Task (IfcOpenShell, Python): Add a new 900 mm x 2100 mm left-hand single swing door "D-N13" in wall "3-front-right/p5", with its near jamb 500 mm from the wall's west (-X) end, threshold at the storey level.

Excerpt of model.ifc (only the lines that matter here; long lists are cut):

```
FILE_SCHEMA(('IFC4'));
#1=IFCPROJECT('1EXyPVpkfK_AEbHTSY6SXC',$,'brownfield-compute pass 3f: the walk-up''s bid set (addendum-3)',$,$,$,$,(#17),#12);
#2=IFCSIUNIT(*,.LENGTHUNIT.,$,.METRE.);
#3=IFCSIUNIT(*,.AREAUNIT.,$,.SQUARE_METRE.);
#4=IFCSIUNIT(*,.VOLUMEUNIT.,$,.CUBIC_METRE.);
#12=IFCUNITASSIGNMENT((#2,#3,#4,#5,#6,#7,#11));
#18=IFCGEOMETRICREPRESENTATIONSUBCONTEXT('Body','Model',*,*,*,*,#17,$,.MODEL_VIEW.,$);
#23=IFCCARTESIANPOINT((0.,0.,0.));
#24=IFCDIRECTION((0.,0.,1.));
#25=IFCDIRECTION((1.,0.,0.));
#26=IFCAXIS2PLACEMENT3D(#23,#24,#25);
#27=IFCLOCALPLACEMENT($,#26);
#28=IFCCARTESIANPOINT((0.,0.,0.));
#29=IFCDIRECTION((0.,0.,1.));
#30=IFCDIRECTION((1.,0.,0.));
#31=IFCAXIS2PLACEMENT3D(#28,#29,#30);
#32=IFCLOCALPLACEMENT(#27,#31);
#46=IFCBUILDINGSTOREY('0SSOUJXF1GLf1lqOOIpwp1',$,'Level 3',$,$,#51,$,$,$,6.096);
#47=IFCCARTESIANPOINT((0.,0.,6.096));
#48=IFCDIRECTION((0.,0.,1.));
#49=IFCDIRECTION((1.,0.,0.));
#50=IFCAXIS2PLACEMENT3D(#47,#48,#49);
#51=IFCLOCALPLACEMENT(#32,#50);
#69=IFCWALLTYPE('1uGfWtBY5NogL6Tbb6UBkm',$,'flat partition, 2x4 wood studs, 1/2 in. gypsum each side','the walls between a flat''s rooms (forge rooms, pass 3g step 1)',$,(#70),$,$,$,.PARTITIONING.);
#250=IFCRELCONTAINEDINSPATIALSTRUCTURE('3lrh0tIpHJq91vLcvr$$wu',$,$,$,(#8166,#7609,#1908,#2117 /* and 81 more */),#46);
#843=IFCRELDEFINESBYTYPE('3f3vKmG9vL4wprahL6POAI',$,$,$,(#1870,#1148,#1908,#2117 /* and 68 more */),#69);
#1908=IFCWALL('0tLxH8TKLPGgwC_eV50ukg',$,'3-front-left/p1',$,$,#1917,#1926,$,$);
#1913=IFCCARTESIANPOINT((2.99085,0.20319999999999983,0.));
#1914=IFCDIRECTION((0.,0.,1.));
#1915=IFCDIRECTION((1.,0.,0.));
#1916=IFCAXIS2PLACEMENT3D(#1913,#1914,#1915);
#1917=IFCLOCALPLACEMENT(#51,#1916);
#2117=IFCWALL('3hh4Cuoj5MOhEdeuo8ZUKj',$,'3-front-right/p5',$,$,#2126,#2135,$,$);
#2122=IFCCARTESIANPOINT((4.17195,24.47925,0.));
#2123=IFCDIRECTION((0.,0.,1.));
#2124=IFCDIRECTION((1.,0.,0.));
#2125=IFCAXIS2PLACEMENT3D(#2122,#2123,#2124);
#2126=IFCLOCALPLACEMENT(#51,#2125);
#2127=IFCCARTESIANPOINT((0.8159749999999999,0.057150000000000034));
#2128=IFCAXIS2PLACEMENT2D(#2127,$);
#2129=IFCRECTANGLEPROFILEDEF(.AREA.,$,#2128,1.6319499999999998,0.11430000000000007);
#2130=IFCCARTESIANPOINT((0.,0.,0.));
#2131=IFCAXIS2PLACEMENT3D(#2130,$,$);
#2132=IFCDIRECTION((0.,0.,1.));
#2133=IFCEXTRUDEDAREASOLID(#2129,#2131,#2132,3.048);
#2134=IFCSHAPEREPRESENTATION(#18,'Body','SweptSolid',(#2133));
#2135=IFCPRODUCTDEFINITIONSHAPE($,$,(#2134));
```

```python
import numpy as np
import ifcopenshell
import ifcopenshell.api.feature
import ifcopenshell.api.geometry
import ifcopenshell.api.root
import ifcopenshell.api.spatial
import ifcopenshell.geom
import ifcopenshell.util.element
import ifcopenshell.util.placement
import ifcopenshell.util.representation
import ifcopenshell.util.shape
import ifcopenshell.util.unit

model = ifcopenshell.open("model.ifc")
unit_scale = ifcopenshell.util.unit.calculate_unit_scale(model)
settings = ifcopenshell.geom.settings()


def volume(element):
    """Net volume in cubic metres, openings subtracted."""
    shape = ifcopenshell.geom.create_shape(settings, element)
    return ifcopenshell.util.shape.get_volume(shape.geometry)


wall = model.by_guid("3hh4Cuoj5MOhEdeuo8ZUKj")
storey = ifcopenshell.util.element.get_container(wall, ifc_class="IfcBuildingStorey")
context = ifcopenshell.util.representation.get_context(model, "Model", "Body", "MODEL_VIEW")
before = volume(wall)

width, height, from_end, sill = 0.9, 2.1, 0.5, 0.0  # metres

# The wall runs along its own X axis, and the end named is its -X end.
wall_shape = ifcopenshell.geom.create_shape(settings, wall)
x, y, z = ifcopenshell.util.shape.get_vertices(wall_shape.geometry).T
start = x.min() + from_end
face, thickness = float(y.min()), float(y.max() - y.min())
wall_matrix = ifcopenshell.util.placement.get_local_placement(wall.ObjectPlacement)
level = ifcopenshell.util.placement.get_local_placement(storey.ObjectPlacement)[2, 3]


def in_wall(x, y):
    """Placement at x, y metres in the wall's axes, at sill height."""
    matrix = wall_matrix.copy()
    matrix[:, 3] = wall_matrix @ np.array([x / unit_scale, y / unit_scale, 0.0, 1.0])
    matrix[2, 3] = level + sill / unit_scale
    return matrix


# Opening: a box that overshoots both wall faces by 50 mm.
opening = ifcopenshell.api.root.create_entity(model, ifc_class="IfcOpeningElement", predefined_type="OPENING")
box = ifcopenshell.api.geometry.add_wall_representation(
    model, context=context, length=width, height=height, thickness=thickness + 0.1
)
ifcopenshell.api.geometry.assign_representation(model, product=opening, representation=box)
ifcopenshell.api.geometry.edit_object_placement(model, product=opening, matrix=in_wall(start, face - 0.05), is_si=False)
ifcopenshell.api.feature.add_feature(model, feature=opening, element=wall)

door = ifcopenshell.api.root.create_entity(model, ifc_class="IfcDoor", name="D-N13", predefined_type="DOOR")
door.OverallWidth, door.OverallHeight = width / unit_scale, height / unit_scale
door.OperationType = "SINGLE_SWING_LEFT"
body = ifcopenshell.api.geometry.add_door_representation(
    model,
    context=context,
    overall_width=door.OverallWidth,
    overall_height=door.OverallHeight,
    operation_type="SINGLE_SWING_LEFT",
    lining_properties={"LiningDepth": thickness / unit_scale, "ThresholdDepth": thickness / unit_scale},
)
ifcopenshell.api.geometry.assign_representation(model, product=door, representation=body)
ifcopenshell.api.spatial.assign_container(model, products=[door], relating_structure=storey)
ifcopenshell.api.feature.add_filling(model, opening=opening, element=door)

# The lining spans the wall, so the door starts at the wall face.
ifcopenshell.api.geometry.edit_object_placement(model, product=door, matrix=in_wall(start, face), is_si=False)

after = volume(wall)

print(f"wall volume {before:.3f} -> {after:.3f} m3")

model.write("model_v2.ifc")
```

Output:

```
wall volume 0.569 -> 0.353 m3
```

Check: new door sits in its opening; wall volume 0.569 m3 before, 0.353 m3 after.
